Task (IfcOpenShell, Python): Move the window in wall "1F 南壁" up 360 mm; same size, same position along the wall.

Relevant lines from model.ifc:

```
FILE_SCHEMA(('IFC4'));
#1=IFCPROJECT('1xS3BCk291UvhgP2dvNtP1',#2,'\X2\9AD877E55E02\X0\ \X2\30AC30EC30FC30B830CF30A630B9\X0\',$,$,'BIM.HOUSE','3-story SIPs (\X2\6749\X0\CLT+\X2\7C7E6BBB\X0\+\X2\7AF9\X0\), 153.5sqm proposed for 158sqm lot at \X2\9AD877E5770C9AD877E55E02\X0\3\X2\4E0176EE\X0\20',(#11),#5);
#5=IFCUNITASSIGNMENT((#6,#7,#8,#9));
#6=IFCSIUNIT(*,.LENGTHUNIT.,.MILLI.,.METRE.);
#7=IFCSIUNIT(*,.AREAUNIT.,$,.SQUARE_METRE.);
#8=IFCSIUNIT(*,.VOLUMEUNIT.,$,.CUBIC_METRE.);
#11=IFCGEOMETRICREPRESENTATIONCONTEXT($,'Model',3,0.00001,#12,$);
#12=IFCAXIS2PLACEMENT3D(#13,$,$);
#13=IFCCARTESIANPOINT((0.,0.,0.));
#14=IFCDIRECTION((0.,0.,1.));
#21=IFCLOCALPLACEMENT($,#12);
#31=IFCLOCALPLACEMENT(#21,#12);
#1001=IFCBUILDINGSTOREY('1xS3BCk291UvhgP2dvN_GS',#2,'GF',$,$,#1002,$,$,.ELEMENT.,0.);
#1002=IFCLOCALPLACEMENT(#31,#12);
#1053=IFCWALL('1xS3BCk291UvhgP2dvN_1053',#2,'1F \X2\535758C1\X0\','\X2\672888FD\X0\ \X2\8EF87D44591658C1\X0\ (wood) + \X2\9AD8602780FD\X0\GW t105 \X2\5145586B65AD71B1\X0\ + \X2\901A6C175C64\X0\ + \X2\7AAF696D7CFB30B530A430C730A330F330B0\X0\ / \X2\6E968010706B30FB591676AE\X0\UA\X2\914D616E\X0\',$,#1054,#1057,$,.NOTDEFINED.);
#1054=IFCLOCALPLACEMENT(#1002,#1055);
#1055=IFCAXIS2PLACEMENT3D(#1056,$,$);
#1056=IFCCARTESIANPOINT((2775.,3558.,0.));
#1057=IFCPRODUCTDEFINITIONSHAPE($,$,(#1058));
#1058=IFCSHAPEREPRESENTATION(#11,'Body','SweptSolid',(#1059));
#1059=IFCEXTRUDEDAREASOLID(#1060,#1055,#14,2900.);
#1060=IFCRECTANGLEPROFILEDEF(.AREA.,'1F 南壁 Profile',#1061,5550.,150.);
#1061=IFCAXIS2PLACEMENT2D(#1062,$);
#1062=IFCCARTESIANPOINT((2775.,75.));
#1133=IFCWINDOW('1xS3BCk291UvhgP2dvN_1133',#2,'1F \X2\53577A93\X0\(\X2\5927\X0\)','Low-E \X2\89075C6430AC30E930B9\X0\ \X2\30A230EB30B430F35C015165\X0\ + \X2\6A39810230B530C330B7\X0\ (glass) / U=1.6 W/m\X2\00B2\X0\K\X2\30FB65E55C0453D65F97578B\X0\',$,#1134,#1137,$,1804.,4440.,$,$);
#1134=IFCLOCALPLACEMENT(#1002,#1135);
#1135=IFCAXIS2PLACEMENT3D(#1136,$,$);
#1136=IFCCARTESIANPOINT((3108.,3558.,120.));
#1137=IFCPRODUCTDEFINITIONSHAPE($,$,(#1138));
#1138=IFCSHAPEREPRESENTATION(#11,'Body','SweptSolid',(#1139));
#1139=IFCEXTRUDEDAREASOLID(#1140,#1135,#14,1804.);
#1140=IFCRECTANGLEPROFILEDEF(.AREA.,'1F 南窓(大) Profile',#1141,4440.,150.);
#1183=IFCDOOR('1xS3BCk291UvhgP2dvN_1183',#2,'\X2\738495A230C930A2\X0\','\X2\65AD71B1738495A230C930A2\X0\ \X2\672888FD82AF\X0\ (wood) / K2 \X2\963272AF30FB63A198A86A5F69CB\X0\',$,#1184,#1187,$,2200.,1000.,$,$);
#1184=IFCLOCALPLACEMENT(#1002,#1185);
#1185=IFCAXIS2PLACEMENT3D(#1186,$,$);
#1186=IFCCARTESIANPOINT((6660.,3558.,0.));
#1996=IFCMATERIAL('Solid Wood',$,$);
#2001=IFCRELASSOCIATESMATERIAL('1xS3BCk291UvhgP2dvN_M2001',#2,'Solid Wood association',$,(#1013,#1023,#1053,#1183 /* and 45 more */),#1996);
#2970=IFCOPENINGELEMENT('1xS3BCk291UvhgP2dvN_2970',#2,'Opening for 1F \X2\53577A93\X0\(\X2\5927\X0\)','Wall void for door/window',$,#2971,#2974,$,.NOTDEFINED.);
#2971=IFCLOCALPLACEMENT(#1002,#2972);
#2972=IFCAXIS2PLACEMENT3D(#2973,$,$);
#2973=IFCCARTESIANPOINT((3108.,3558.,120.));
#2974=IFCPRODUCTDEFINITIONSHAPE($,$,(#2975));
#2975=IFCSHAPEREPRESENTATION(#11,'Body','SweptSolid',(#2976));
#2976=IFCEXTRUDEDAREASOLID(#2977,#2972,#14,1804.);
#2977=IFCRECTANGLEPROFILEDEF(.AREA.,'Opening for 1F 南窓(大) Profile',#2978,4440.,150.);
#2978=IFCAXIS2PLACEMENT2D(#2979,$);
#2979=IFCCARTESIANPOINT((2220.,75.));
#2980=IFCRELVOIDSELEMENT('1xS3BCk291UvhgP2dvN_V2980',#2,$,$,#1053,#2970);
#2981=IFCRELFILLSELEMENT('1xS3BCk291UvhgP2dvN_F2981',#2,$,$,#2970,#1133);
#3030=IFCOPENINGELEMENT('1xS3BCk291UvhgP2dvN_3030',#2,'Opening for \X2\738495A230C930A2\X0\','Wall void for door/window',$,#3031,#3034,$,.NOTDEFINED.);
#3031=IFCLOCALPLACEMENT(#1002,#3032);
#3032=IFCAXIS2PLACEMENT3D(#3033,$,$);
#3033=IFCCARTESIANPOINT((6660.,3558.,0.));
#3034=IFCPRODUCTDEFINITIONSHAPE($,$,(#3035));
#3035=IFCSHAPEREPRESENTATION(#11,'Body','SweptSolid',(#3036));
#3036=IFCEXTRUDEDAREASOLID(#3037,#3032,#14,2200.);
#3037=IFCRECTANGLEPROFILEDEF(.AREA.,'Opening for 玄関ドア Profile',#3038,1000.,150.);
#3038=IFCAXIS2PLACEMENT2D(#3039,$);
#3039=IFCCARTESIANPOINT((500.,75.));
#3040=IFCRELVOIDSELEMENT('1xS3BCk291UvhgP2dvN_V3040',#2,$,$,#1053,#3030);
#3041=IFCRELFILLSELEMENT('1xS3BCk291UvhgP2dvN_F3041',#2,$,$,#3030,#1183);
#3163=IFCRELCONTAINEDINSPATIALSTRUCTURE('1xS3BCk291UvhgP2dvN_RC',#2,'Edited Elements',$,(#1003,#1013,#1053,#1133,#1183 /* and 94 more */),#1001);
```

```python
import numpy as np
import ifcopenshell
import ifcopenshell.api.geometry
import ifcopenshell.util.placement
import ifcopenshell.util.unit

model = ifcopenshell.open("model.ifc")
unit_scale = ifcopenshell.util.unit.calculate_unit_scale(model)

window = model.by_guid("1xS3BCk291UvhgP2dvN_1133")
opening = window.FillsVoids[0].RelatingOpeningElement
dz = 0.36 / unit_scale

shift = np.array([0.0, 0.0, dz])
# The window is not placed relative to its opening, so move both.
for product in (opening, window):
    matrix = ifcopenshell.util.placement.get_local_placement(product.ObjectPlacement)
    matrix[:3, 3] += shift
    ifcopenshell.api.geometry.edit_object_placement(model, product=product, matrix=matrix, is_si=False)

print(f"moved by {dz * unit_scale:+.3f} m")

model.write("model_updated.ifc")
```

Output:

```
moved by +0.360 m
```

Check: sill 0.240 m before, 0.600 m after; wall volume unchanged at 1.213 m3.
